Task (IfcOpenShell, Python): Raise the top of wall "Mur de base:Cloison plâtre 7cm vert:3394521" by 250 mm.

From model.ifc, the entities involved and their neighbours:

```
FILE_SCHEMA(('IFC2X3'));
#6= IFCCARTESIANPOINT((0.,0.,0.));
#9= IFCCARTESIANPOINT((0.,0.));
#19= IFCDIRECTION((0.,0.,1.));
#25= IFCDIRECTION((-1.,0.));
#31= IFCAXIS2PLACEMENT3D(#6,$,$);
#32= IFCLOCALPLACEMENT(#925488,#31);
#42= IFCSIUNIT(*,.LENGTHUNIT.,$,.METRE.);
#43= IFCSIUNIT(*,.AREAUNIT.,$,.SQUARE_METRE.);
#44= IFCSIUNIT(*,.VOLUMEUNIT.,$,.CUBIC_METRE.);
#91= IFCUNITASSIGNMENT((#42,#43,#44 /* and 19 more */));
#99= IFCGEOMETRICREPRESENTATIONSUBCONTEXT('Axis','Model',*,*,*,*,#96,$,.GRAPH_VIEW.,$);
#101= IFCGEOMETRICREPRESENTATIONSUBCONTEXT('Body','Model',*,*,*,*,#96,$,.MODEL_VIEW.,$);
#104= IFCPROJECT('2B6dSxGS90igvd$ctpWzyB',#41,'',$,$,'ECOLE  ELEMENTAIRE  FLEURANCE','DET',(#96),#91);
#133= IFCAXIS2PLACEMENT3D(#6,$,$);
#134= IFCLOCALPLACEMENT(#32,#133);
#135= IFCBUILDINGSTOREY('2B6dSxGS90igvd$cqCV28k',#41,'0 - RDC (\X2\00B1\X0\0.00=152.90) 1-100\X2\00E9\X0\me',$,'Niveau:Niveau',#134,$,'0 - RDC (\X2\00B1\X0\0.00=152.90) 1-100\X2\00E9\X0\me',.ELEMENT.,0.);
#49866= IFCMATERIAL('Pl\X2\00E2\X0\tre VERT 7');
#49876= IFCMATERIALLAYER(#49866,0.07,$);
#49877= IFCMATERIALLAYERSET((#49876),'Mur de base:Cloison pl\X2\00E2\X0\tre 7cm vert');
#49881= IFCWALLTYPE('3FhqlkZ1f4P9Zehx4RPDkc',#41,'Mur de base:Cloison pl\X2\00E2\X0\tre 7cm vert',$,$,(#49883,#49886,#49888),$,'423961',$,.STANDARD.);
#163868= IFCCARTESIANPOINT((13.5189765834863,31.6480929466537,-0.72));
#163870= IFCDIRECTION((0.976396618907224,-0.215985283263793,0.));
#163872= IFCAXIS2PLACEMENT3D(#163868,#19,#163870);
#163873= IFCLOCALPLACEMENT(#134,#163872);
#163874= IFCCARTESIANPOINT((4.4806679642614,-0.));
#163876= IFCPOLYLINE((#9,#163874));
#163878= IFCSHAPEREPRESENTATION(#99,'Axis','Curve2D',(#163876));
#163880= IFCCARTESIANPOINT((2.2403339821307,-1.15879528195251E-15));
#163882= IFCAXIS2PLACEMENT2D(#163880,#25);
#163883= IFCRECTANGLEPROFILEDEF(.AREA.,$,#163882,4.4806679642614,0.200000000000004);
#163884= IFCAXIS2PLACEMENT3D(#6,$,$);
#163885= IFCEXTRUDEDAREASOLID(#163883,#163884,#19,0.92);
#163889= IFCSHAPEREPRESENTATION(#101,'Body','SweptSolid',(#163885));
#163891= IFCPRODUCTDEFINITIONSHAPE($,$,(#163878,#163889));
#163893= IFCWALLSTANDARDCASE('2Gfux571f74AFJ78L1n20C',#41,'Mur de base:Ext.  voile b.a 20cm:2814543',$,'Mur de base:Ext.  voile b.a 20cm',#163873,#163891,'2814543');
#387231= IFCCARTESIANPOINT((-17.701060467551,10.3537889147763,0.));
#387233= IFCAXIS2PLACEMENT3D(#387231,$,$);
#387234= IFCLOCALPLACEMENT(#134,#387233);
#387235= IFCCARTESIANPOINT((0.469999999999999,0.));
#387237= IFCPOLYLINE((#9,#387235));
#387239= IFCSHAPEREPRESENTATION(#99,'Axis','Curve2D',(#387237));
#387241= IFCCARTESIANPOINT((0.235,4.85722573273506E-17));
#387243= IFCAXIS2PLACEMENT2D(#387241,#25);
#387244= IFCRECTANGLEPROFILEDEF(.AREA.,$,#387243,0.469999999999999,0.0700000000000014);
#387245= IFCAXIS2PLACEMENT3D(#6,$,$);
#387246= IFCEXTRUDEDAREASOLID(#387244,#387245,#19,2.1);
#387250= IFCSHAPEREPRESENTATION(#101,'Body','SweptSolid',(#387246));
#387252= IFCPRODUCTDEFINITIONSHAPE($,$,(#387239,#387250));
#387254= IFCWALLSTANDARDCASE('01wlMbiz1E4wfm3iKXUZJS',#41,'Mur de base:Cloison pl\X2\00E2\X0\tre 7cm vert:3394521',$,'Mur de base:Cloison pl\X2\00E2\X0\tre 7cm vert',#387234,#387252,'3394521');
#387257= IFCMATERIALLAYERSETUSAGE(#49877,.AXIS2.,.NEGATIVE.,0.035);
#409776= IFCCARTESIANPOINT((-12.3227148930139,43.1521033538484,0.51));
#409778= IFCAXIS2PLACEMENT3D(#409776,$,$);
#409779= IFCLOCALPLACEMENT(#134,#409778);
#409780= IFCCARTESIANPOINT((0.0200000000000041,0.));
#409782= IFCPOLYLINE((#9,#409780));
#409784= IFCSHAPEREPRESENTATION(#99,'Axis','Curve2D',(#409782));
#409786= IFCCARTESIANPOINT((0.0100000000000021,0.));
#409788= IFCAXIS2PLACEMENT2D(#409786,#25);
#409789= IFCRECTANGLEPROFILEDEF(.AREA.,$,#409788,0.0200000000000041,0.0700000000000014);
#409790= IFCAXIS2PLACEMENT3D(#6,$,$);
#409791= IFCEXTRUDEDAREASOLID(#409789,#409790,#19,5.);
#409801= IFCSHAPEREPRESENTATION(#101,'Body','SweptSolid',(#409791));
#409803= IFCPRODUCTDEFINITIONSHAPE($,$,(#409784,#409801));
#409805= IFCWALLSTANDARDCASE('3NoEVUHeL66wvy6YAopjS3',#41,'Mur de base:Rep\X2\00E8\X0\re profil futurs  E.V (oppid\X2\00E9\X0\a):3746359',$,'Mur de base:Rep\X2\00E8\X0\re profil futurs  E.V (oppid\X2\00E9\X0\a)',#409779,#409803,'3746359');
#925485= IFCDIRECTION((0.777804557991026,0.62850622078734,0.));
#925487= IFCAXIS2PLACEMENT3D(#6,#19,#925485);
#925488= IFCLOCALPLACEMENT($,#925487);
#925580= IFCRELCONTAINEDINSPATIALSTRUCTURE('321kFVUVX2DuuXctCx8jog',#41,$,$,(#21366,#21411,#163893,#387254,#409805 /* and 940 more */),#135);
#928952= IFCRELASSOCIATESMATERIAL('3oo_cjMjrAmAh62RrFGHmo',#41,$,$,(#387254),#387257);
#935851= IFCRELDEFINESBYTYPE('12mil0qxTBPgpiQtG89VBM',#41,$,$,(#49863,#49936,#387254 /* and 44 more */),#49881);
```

```python
import ifcopenshell
import ifcopenshell.geom
import ifcopenshell.util.representation
import ifcopenshell.util.shape
import ifcopenshell.util.unit

model = ifcopenshell.open("model.ifc")
unit_scale = ifcopenshell.util.unit.calculate_unit_scale(model)
settings = ifcopenshell.geom.settings()


def volume(element):
    """Net volume in cubic metres, openings subtracted."""
    shape = ifcopenshell.geom.create_shape(settings, element)
    return ifcopenshell.util.shape.get_volume(shape.geometry)


wall = model.by_guid("01wlMbiz1E4wfm3iKXUZJS")
before = volume(wall)

body = ifcopenshell.util.representation.get_representation(wall, "Model", "Body")
solid = body.Items[0]
old_height = solid.Depth
solid.Depth += 0.25 / unit_scale
after = volume(wall)

print(f"height {old_height:g} -> {solid.Depth:g}, volume {before:.3f} -> {after:.3f} m3")

model.write("model_updated.ifc")
```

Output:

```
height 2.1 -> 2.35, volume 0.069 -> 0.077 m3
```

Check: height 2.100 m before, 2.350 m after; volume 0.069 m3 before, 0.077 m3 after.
